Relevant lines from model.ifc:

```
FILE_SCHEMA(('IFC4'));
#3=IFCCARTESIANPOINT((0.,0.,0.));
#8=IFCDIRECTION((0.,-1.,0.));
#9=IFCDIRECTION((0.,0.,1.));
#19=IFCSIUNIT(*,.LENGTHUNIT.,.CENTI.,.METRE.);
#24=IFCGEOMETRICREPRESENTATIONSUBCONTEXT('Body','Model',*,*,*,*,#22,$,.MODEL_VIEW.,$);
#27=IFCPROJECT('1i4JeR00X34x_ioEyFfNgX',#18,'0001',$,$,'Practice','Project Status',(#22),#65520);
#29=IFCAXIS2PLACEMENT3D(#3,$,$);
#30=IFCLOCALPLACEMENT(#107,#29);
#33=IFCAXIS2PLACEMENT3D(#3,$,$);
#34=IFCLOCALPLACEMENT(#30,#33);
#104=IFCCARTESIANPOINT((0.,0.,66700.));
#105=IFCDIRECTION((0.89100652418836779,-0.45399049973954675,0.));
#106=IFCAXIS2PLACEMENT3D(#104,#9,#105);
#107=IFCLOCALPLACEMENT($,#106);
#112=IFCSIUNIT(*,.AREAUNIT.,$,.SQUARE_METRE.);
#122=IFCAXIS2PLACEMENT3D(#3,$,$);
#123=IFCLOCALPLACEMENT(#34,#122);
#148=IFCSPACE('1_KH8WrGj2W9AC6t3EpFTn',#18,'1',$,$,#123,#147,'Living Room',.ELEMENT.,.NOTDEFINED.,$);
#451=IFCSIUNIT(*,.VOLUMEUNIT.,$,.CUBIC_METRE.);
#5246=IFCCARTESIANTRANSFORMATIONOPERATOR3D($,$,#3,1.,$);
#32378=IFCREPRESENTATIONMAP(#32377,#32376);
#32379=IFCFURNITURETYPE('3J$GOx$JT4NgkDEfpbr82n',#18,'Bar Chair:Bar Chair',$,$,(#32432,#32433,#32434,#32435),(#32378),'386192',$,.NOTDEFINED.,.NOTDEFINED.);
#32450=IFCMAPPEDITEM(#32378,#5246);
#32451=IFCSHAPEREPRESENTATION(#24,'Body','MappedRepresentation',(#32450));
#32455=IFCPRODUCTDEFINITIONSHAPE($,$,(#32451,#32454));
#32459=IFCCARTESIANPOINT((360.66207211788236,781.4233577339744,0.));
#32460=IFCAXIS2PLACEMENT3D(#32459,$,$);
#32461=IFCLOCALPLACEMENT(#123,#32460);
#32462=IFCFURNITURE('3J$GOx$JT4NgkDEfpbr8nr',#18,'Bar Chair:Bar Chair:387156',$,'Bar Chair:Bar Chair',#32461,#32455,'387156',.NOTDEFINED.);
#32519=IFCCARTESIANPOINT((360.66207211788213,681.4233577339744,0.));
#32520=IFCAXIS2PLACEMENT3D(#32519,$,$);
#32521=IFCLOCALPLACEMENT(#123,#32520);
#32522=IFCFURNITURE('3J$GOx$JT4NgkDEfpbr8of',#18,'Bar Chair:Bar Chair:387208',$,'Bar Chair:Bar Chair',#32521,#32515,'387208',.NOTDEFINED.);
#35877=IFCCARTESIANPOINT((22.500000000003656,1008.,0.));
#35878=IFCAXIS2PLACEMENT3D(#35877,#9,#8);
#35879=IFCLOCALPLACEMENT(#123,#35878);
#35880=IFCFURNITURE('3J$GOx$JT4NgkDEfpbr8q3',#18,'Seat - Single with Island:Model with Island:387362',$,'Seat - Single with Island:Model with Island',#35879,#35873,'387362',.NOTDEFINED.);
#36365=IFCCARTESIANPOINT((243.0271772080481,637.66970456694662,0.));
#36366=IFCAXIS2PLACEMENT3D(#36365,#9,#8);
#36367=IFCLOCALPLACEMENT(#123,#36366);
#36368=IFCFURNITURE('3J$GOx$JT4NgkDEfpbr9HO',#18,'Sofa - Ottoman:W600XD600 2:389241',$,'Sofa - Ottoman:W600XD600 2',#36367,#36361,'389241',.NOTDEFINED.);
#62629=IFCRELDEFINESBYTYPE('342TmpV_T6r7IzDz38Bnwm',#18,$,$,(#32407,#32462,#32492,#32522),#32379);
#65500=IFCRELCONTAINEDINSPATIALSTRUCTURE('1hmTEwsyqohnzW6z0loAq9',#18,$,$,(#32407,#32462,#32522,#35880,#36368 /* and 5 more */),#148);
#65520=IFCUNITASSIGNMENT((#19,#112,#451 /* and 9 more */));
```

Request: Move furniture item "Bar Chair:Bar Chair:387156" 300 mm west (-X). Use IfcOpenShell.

```python
import ifcopenshell
import ifcopenshell.api.geometry
import ifcopenshell.util.placement
import ifcopenshell.util.unit

model = ifcopenshell.open("model.ifc")
unit_scale = ifcopenshell.util.unit.calculate_unit_scale(model)

item = model.by_guid("3J$GOx$JT4NgkDEfpbr8nr")
matrix = ifcopenshell.util.placement.get_local_placement(item.ObjectPlacement)
matrix[0, 3] -= 0.3 / unit_scale
ifcopenshell.api.geometry.edit_object_placement(model, product=item, matrix=matrix, is_si=False)

print(ifcopenshell.util.placement.get_local_placement(item.ObjectPlacement).round(3) + 0.0)

model.write("model_v2.ifc")
```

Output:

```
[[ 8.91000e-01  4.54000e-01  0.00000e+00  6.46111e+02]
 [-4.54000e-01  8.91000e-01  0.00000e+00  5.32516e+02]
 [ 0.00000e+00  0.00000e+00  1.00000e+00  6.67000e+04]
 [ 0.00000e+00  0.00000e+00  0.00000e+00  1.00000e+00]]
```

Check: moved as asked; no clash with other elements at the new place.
